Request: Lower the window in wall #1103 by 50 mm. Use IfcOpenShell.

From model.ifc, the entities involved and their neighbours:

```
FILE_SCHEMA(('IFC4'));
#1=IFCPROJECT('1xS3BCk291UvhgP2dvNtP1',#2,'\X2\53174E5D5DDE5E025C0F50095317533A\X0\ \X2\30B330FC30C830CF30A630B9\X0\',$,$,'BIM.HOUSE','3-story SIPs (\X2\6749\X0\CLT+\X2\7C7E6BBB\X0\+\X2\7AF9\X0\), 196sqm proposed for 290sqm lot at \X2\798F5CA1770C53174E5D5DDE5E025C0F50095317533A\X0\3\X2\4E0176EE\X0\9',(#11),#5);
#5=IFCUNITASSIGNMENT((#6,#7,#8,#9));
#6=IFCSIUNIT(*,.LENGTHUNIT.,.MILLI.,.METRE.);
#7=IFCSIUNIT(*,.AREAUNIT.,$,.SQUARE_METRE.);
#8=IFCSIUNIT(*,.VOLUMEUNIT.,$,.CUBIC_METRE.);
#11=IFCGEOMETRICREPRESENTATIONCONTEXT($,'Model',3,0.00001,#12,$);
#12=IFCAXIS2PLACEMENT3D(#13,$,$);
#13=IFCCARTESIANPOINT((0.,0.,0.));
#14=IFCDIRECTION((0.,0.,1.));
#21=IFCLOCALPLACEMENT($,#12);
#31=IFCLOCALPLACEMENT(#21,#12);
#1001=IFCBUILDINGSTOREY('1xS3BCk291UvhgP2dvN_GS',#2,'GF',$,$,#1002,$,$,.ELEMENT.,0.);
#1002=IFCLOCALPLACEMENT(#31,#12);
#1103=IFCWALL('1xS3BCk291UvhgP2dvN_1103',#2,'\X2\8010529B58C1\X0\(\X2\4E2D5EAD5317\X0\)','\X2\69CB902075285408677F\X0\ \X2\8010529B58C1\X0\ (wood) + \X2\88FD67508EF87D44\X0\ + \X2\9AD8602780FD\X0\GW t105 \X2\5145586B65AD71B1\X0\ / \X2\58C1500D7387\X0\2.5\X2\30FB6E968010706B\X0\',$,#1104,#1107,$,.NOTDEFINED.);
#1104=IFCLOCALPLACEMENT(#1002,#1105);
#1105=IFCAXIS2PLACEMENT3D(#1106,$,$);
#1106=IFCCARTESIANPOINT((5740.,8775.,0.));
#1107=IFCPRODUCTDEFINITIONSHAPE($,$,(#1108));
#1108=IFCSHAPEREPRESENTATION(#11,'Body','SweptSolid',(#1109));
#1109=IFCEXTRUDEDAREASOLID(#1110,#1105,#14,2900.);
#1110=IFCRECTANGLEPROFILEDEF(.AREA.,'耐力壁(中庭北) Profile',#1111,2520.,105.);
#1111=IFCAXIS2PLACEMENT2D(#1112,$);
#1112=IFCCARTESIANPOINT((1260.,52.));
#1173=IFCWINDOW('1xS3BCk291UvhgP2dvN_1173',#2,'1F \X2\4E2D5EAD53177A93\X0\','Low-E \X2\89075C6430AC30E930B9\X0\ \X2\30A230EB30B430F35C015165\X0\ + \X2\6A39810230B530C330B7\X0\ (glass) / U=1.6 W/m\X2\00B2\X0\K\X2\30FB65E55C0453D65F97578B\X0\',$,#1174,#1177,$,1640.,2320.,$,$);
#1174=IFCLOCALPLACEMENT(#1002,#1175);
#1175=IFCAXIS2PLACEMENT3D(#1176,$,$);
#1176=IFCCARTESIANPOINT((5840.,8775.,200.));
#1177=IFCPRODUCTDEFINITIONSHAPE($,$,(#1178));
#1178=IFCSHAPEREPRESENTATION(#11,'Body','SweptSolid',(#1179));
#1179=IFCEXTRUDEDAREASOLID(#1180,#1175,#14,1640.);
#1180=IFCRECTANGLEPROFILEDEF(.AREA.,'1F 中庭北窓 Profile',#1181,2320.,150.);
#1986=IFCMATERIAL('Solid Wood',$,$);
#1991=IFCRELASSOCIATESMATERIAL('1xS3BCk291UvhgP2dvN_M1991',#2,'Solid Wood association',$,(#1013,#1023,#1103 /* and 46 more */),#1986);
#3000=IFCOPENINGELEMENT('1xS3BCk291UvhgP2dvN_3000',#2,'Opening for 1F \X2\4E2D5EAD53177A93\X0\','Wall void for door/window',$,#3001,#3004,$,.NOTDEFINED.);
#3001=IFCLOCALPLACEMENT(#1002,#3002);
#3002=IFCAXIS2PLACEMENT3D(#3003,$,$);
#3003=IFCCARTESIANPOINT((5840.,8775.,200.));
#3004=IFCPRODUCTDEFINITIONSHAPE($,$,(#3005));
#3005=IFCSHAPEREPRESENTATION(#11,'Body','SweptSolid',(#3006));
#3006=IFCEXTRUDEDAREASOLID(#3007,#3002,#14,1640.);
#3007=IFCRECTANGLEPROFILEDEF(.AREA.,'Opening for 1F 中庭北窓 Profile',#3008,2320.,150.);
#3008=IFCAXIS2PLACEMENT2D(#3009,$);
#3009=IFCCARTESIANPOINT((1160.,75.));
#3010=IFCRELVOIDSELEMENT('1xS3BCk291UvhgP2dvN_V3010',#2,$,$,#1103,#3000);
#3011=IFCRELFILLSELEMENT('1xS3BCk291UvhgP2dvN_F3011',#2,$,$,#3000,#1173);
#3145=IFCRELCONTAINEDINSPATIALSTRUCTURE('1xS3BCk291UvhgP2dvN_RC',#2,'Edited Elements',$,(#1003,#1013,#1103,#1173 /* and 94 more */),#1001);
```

```python
import numpy as np
import ifcopenshell
import ifcopenshell.api.geometry
import ifcopenshell.util.placement
import ifcopenshell.util.unit

model = ifcopenshell.open("model.ifc")
unit_scale = ifcopenshell.util.unit.calculate_unit_scale(model)

window = model.by_id(1173)
opening = window.FillsVoids[0].RelatingOpeningElement
dz = -0.05 / unit_scale

shift = np.array([0.0, 0.0, dz])
# The window is not placed relative to its opening, so move both.
for product in (opening, window):
    matrix = ifcopenshell.util.placement.get_local_placement(product.ObjectPlacement)
    matrix[:3, 3] += shift
    ifcopenshell.api.geometry.edit_object_placement(model, product=product, matrix=matrix, is_si=False)

print(f"moved by {dz * unit_scale:+.3f} m")

model.write("model_edited.ifc")
```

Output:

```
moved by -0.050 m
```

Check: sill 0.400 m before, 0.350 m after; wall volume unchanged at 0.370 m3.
